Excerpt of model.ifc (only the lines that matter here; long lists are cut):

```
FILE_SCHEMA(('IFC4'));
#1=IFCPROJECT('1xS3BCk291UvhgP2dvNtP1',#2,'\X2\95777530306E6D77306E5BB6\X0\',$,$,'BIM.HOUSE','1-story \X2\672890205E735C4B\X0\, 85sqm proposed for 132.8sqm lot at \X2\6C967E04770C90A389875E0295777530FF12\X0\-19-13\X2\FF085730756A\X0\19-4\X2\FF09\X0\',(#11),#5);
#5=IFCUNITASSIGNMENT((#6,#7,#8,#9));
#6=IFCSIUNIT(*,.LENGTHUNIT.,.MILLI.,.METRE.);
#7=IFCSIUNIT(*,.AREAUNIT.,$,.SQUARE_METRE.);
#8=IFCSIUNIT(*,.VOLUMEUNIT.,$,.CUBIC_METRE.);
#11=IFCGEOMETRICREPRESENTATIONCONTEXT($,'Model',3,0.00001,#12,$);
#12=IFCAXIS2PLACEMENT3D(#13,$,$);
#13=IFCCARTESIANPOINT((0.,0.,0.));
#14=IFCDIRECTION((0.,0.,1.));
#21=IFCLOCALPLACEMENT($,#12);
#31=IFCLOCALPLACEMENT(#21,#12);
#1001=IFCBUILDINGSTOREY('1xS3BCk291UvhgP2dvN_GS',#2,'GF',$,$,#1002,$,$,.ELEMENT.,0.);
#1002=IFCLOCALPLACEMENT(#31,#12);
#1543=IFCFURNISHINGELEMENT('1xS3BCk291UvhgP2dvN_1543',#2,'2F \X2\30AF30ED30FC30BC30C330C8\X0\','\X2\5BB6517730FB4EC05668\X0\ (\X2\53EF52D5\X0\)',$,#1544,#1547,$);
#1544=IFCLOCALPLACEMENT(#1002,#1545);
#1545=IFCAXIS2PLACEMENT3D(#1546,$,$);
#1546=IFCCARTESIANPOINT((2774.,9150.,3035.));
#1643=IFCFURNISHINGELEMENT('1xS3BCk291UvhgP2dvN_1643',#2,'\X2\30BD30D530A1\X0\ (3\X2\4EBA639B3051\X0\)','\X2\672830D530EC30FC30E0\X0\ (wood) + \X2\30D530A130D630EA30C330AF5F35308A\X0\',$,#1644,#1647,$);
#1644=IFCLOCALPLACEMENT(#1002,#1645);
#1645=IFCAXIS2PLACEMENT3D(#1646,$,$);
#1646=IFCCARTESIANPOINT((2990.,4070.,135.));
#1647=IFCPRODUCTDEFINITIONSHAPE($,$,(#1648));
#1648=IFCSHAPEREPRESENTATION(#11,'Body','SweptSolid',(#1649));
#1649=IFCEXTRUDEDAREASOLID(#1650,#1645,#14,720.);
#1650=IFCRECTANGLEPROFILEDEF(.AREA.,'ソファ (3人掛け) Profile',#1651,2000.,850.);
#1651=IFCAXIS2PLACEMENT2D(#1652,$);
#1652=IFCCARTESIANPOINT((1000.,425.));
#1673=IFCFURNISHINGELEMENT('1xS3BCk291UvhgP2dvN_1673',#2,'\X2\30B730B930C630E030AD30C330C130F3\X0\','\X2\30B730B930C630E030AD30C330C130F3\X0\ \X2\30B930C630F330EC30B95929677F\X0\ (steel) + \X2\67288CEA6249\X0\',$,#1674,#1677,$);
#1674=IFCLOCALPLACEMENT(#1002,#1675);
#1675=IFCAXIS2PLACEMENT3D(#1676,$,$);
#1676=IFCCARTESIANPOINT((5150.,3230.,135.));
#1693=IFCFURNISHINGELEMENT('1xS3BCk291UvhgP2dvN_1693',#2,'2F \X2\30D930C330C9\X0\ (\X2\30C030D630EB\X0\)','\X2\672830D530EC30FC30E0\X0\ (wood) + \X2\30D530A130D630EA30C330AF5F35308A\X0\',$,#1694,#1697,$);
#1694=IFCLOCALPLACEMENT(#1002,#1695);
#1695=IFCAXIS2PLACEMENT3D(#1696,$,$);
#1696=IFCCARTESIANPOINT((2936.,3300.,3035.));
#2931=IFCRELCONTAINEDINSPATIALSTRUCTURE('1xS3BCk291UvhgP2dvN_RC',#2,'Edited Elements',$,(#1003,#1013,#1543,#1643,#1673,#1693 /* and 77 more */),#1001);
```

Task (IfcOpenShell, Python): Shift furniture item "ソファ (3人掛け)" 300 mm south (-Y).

```python
import ifcopenshell
import ifcopenshell.api.geometry
import ifcopenshell.util.placement

model = ifcopenshell.open("model.ifc")

item = model.by_id(1643)
matrix = ifcopenshell.util.placement.get_local_placement(item.ObjectPlacement)
matrix[1, 3] -= 300.0
ifcopenshell.api.geometry.edit_object_placement(model, product=item, matrix=matrix, is_si=False)

print(ifcopenshell.util.placement.get_local_placement(item.ObjectPlacement).round(3) + 0.0)

model.write("model_edited.ifc")
```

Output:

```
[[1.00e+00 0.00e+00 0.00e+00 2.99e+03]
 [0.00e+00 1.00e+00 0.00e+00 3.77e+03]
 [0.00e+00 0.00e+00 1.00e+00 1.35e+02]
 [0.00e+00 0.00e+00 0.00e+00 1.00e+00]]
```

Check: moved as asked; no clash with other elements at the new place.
